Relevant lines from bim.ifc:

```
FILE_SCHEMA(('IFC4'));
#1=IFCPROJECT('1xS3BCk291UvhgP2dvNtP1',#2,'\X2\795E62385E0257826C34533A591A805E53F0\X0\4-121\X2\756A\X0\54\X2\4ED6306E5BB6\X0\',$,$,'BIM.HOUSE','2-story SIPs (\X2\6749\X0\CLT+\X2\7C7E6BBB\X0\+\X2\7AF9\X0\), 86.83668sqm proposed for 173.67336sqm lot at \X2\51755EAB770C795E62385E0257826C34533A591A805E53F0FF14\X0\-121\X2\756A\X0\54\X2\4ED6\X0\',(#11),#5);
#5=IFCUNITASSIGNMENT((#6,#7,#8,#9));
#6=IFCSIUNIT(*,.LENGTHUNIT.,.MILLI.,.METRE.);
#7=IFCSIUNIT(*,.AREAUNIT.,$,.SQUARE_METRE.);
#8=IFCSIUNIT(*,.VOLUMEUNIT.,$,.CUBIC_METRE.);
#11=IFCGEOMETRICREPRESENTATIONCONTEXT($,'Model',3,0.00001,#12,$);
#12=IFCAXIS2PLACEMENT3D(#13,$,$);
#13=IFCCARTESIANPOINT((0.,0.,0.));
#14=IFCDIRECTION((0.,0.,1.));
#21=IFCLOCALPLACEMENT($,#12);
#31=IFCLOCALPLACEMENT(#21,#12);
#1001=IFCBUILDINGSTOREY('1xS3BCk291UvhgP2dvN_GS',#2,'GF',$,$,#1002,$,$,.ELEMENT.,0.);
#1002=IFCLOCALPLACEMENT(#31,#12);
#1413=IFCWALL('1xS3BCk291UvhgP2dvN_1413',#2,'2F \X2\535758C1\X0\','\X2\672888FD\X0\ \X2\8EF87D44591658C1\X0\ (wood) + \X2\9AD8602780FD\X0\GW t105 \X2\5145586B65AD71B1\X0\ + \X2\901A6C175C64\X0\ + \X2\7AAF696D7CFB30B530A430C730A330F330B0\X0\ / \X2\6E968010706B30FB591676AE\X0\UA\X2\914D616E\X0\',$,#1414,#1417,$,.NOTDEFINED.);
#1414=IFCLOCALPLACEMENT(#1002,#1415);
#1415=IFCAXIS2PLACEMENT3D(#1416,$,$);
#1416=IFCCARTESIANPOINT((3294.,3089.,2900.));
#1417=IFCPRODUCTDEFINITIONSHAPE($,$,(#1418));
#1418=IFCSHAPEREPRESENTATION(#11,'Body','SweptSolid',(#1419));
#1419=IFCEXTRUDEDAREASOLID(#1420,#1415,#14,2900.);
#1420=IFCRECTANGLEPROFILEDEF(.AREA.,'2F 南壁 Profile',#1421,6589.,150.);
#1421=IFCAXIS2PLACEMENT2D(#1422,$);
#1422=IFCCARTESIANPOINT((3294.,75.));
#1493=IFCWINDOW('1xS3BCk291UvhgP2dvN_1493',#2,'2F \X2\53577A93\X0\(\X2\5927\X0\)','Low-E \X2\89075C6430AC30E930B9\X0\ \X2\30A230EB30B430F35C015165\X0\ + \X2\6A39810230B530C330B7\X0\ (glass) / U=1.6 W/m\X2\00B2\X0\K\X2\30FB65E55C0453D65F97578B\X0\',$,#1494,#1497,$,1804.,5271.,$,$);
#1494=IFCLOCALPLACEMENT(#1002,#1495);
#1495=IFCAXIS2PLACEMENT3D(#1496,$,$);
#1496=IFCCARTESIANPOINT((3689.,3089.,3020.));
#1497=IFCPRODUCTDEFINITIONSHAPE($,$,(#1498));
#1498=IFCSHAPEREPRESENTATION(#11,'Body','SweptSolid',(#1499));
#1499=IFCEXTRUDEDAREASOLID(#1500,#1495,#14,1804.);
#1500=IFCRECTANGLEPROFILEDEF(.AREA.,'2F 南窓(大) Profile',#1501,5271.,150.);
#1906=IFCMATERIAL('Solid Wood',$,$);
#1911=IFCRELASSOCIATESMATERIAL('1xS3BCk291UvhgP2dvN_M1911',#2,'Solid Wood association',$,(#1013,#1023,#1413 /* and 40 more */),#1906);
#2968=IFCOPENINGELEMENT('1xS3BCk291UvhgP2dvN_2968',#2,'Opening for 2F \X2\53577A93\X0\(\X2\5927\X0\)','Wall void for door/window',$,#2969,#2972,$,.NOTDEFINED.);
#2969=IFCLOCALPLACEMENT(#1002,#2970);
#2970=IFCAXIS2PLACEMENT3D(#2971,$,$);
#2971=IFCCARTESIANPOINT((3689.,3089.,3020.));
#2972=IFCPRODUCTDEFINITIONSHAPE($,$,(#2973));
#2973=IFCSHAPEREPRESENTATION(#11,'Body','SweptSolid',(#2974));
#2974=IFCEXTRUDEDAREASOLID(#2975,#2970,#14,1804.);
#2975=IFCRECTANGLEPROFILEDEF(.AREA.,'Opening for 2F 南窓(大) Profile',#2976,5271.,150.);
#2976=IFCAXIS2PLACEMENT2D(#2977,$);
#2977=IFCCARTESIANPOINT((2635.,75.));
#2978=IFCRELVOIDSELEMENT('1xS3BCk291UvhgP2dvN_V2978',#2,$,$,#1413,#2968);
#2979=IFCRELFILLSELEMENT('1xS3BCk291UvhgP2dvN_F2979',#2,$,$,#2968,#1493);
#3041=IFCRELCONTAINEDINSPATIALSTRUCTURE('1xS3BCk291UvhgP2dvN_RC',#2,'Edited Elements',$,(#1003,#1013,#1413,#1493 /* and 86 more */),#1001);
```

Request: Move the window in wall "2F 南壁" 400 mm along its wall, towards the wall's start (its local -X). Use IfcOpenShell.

```python
import ifcopenshell
import ifcopenshell.api.geometry
import ifcopenshell.util.placement
import ifcopenshell.util.unit

model = ifcopenshell.open("bim.ifc")
unit_scale = ifcopenshell.util.unit.calculate_unit_scale(model)

window = model.by_id(1493)
opening = window.FillsVoids[0].RelatingOpeningElement
wall = opening.VoidsElements[0].RelatingBuildingElement

wall_matrix = ifcopenshell.util.placement.get_local_placement(wall.ObjectPlacement)
shift = wall_matrix[:3, 0] * -0.4 / unit_scale
before = ifcopenshell.util.placement.get_local_placement(window.ObjectPlacement)[:3, 3].copy()

# The window is not placed relative to its opening, so move both.
for product in (opening, window):
    matrix = ifcopenshell.util.placement.get_local_placement(product.ObjectPlacement)
    matrix[:3, 3] += shift
    ifcopenshell.api.geometry.edit_object_placement(model, product=product, matrix=matrix, is_si=False)

after = ifcopenshell.util.placement.get_local_placement(window.ObjectPlacement)[:3, 3]
print("window moved by", (after - before).round(3) + 0.0)

model.write("bim_updated.ifc")
```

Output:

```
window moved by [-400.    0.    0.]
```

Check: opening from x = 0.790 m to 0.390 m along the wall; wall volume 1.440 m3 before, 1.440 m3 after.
